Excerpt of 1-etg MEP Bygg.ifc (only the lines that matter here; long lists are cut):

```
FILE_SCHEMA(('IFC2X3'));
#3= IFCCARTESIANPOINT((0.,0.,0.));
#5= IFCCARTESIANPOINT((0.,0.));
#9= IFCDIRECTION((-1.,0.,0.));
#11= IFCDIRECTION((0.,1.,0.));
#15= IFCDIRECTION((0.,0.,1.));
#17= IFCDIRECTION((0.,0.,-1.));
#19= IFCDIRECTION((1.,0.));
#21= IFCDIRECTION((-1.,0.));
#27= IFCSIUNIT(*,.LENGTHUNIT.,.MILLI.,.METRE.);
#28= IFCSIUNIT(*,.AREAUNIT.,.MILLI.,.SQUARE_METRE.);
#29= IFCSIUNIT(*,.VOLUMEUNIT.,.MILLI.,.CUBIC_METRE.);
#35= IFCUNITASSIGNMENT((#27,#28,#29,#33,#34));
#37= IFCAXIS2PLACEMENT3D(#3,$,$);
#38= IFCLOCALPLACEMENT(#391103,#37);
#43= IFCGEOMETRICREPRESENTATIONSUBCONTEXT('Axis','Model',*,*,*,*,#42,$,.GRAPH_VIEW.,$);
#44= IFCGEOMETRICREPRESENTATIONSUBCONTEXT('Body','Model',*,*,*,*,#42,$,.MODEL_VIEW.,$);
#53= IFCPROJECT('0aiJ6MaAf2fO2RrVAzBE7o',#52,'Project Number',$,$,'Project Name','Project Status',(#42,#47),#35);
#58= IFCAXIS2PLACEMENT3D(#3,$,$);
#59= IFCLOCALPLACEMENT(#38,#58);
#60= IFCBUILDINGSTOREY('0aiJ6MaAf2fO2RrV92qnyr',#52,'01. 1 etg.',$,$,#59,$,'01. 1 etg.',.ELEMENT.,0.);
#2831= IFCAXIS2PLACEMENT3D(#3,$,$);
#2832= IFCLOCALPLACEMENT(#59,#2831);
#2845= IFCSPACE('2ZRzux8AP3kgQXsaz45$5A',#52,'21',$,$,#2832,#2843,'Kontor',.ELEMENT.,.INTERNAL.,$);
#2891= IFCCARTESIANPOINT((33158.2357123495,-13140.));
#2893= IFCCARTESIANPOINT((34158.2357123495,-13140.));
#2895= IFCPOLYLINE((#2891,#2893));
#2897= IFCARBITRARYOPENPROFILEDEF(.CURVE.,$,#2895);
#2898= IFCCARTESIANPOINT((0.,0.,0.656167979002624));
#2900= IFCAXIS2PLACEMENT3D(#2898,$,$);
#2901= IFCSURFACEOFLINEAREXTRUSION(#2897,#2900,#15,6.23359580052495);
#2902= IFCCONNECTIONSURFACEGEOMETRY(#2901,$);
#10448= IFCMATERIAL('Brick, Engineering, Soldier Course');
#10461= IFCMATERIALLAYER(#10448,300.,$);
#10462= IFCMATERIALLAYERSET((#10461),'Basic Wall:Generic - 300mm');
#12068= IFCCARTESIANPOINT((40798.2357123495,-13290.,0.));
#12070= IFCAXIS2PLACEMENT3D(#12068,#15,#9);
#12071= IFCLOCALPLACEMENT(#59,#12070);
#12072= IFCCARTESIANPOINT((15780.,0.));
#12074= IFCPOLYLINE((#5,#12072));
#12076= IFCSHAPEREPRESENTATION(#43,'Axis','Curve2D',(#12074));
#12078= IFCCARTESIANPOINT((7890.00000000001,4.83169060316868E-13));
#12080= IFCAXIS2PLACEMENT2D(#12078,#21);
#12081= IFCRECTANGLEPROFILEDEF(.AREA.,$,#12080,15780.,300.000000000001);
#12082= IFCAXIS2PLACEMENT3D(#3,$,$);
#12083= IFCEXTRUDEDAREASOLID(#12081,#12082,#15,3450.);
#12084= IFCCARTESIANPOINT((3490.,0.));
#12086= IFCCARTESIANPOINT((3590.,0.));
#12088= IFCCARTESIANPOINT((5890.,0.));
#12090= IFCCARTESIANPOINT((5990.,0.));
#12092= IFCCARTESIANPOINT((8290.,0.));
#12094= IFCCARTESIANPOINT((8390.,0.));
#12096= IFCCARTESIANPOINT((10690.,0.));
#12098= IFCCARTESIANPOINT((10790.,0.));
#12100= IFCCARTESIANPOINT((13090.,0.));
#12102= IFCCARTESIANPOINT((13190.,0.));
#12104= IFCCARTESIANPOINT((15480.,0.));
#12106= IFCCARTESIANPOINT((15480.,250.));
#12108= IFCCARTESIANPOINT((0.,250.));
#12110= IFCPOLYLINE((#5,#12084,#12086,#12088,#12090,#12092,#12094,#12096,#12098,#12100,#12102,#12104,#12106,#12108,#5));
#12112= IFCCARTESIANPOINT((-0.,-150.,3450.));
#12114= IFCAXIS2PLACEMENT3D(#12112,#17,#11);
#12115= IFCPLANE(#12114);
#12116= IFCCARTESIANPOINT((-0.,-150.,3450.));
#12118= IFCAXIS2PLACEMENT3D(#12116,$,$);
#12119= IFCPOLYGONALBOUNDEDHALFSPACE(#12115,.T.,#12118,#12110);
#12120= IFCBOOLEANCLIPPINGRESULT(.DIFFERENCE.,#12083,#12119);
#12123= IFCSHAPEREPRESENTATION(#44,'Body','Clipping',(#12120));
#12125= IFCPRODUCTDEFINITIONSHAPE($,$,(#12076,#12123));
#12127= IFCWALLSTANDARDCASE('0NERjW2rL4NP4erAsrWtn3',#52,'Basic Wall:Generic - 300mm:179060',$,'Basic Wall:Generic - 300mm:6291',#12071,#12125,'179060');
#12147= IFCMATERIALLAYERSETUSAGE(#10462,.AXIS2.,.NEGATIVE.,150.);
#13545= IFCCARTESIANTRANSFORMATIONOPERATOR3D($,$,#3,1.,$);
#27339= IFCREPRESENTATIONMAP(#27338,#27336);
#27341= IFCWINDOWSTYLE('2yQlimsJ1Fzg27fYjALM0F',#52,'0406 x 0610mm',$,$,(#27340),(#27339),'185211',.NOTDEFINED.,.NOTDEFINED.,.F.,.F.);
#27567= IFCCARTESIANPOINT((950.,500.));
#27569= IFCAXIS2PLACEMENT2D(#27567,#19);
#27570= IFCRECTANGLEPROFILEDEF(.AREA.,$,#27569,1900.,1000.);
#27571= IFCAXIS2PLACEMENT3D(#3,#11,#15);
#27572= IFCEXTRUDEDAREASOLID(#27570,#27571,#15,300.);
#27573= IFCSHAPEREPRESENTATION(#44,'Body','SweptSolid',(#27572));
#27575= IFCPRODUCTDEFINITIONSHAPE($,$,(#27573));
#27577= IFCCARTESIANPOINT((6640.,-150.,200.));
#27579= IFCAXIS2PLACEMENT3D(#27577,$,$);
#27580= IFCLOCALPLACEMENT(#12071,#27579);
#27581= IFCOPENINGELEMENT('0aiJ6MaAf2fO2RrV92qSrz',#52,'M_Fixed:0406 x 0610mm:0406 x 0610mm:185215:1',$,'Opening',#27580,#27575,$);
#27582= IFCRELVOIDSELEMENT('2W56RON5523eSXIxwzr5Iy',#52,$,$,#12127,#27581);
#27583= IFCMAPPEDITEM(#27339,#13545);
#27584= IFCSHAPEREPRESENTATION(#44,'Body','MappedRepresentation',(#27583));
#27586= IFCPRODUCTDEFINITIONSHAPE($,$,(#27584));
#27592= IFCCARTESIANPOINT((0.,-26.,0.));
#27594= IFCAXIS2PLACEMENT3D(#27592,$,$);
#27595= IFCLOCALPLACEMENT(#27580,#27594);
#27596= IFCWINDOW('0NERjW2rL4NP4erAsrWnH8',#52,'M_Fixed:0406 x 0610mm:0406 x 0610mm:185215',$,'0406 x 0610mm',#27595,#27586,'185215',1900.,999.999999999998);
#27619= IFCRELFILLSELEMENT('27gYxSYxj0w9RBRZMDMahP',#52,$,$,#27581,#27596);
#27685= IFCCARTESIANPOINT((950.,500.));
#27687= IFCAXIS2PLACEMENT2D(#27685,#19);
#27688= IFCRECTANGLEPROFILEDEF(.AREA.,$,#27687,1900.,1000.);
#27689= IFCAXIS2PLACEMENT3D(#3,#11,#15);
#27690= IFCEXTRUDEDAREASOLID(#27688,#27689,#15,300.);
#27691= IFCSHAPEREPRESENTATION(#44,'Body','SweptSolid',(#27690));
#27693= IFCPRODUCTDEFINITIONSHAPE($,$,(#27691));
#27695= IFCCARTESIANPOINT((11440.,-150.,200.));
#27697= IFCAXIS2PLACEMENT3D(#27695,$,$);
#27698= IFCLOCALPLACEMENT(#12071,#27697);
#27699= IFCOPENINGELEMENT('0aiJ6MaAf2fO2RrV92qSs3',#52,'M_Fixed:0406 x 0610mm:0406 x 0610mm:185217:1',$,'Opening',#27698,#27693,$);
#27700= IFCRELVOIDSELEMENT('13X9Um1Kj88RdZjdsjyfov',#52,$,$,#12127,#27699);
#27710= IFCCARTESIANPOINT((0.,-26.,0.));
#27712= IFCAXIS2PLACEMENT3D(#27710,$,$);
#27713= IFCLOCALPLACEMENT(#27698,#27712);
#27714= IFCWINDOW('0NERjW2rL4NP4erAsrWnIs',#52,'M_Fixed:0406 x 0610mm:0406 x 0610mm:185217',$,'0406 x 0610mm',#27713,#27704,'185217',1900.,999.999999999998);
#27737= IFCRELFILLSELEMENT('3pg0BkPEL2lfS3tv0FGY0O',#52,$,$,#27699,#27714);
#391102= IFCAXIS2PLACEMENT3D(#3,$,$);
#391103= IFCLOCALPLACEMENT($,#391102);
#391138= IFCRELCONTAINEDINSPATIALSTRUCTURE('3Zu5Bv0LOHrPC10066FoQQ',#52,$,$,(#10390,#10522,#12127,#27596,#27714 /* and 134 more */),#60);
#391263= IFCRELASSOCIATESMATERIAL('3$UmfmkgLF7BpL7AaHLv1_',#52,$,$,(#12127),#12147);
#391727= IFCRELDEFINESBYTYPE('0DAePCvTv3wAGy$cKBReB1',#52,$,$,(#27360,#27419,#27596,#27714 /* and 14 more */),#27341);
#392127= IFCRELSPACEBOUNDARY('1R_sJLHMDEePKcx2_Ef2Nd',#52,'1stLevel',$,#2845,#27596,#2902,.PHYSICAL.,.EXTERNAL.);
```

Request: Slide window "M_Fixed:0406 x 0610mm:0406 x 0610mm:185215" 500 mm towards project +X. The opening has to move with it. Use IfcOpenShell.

```python
import numpy as np
import ifcopenshell
import ifcopenshell.api.geometry
import ifcopenshell.util.placement
import ifcopenshell.util.unit

model = ifcopenshell.open("1-etg MEP Bygg.ifc")
unit_scale = ifcopenshell.util.unit.calculate_unit_scale(model)

window = model.by_id(27596)
opening = window.FillsVoids[0].RelatingOpeningElement
wall = opening.VoidsElements[0].RelatingBuildingElement

wall_matrix = ifcopenshell.util.placement.get_local_placement(wall.ObjectPlacement)
shift = wall_matrix[:3, 0] * -0.5 / unit_scale
before = ifcopenshell.util.placement.get_local_placement(window.ObjectPlacement)[:3, 3].copy()

# The window is placed relative to its opening, so it follows when the opening moves.
matrix = ifcopenshell.util.placement.get_local_placement(opening.ObjectPlacement)
matrix[:3, 3] += shift
ifcopenshell.api.geometry.edit_object_placement(
    model, product=opening, matrix=matrix, is_si=False, should_transform_children=True
)

# Space boundary surfaces are stored in each space's coordinates; move them too.
for rel in window.ProvidesBoundaries:
    if not rel.ConnectionGeometry:
        continue
    surface = rel.ConnectionGeometry.SurfaceOnRelatingElement
    space_matrix = ifcopenshell.util.placement.get_local_placement(rel.RelatingSpace.ObjectPlacement)
    point = np.array(surface.Position.Location.Coordinates) + space_matrix[:3, :3].T @ shift
    surface.Position = model.createIfcAxis2Placement3D(
        model.createIfcCartesianPoint(point.tolist()), surface.Position.Axis, surface.Position.RefDirection
    )

after = ifcopenshell.util.placement.get_local_placement(window.ObjectPlacement)[:3, 3]
print("window moved by", (after - before).round(3) + 0.0)

model.write("1-etg MEP Bygg_edited.ifc")
```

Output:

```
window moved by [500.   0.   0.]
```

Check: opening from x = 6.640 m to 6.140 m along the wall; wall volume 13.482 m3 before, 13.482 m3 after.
